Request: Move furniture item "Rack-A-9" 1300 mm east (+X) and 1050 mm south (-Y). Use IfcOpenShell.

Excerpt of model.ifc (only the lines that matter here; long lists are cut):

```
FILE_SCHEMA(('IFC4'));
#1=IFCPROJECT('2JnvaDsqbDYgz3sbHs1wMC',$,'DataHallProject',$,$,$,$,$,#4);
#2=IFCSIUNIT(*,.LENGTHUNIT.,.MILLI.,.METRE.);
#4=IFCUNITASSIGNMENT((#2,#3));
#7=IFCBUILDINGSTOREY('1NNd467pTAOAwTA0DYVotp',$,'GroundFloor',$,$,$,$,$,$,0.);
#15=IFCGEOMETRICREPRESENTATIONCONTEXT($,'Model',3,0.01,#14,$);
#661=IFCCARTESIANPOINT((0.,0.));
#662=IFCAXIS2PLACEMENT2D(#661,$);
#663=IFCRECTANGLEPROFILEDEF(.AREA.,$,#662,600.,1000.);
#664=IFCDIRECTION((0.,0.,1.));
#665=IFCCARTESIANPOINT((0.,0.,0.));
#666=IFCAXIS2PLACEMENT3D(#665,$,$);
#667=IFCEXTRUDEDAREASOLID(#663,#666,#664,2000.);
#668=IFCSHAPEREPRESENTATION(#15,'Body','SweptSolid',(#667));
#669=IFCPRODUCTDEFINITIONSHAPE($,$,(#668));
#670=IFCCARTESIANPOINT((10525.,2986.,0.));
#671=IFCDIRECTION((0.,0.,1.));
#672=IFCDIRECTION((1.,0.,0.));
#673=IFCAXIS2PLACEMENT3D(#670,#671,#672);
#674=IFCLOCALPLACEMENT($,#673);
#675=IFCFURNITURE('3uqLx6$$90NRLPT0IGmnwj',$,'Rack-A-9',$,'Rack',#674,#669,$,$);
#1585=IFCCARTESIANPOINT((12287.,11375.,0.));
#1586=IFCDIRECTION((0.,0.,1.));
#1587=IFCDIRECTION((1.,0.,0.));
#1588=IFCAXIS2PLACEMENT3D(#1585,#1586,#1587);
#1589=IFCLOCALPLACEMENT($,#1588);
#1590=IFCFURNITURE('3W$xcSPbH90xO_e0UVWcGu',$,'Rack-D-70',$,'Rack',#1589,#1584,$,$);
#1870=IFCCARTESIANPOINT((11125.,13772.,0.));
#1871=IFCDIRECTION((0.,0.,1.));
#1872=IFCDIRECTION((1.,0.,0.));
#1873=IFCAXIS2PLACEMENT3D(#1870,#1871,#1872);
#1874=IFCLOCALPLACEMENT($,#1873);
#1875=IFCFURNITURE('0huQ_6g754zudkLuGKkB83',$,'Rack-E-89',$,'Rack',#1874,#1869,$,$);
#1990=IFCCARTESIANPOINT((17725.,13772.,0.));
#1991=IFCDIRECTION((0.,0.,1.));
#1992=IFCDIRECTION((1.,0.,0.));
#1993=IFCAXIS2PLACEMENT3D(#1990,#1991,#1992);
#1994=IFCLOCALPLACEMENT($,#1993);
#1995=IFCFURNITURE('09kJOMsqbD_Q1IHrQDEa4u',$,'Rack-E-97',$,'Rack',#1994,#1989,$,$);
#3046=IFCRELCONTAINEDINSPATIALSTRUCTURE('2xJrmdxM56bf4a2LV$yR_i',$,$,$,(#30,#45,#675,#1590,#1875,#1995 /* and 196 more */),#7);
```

```python
import ifcopenshell
import ifcopenshell.api.geometry
import ifcopenshell.util.placement
import ifcopenshell.util.unit

model = ifcopenshell.open("model.ifc")
unit_scale = ifcopenshell.util.unit.calculate_unit_scale(model)

item = model.by_guid("3uqLx6$$90NRLPT0IGmnwj")
matrix = ifcopenshell.util.placement.get_local_placement(item.ObjectPlacement)
matrix[0, 3] += 1.3 / unit_scale
matrix[1, 3] -= 1.05 / unit_scale
ifcopenshell.api.geometry.edit_object_placement(model, product=item, matrix=matrix, is_si=False)

print(ifcopenshell.util.placement.get_local_placement(item.ObjectPlacement).round(3) + 0.0)

model.write("model_v2.ifc")
```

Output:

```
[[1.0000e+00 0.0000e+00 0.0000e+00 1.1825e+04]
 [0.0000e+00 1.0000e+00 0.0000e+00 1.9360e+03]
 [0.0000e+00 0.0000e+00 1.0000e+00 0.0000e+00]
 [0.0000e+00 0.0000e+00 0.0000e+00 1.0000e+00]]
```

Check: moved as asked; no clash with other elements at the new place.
